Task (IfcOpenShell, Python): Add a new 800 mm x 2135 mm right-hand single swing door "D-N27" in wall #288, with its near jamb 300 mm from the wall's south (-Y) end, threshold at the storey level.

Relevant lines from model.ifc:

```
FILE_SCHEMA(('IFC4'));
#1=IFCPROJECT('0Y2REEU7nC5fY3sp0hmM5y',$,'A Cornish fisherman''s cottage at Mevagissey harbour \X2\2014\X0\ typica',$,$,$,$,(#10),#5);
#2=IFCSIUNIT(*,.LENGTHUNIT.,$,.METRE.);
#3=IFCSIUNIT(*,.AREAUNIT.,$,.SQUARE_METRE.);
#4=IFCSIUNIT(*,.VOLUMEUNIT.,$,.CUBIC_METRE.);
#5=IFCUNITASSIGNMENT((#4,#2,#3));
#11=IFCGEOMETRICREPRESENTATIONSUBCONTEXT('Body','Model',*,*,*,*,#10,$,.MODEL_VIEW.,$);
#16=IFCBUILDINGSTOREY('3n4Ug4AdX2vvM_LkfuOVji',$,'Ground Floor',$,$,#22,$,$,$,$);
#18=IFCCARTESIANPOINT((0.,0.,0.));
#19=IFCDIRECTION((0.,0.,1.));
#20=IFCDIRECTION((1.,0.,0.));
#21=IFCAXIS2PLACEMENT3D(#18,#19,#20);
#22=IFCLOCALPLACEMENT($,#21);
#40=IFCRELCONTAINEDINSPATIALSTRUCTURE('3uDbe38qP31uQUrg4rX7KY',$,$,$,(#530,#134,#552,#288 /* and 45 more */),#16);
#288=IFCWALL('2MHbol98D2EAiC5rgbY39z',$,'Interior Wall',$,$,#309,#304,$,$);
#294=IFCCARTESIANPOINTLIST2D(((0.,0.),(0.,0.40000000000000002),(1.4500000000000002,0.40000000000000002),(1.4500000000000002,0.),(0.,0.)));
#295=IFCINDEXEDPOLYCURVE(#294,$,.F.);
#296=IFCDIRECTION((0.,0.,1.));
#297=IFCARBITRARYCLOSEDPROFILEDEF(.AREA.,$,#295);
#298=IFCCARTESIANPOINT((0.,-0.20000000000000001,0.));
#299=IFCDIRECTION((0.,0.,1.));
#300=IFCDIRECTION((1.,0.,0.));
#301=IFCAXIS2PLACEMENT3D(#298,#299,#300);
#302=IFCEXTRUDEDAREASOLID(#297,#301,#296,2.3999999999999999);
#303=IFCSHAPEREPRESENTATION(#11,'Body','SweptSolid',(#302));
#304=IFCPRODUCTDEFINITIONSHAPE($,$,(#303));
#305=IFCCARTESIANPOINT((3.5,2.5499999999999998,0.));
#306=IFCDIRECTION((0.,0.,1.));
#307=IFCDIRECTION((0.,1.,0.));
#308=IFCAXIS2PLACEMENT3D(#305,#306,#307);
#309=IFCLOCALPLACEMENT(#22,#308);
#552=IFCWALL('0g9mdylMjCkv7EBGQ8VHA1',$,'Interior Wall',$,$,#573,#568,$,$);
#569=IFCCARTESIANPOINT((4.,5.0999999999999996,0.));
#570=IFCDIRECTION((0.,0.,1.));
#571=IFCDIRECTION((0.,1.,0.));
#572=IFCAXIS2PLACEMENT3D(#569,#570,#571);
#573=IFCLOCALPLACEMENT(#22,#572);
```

```python
import numpy as np
import ifcopenshell
import ifcopenshell.api.feature
import ifcopenshell.api.geometry
import ifcopenshell.api.root
import ifcopenshell.api.spatial
import ifcopenshell.geom
import ifcopenshell.util.element
import ifcopenshell.util.placement
import ifcopenshell.util.representation
import ifcopenshell.util.shape
import ifcopenshell.util.unit

model = ifcopenshell.open("model.ifc")
unit_scale = ifcopenshell.util.unit.calculate_unit_scale(model)
settings = ifcopenshell.geom.settings()


def volume(element):
    """Net volume in cubic metres, openings subtracted."""
    shape = ifcopenshell.geom.create_shape(settings, element)
    return ifcopenshell.util.shape.get_volume(shape.geometry)


wall = model.by_guid("2MHbol98D2EAiC5rgbY39z")
storey = ifcopenshell.util.element.get_container(wall, ifc_class="IfcBuildingStorey")
context = ifcopenshell.util.representation.get_context(model, "Model", "Body", "MODEL_VIEW")
before = volume(wall)

width, height, from_end, sill = 0.8, 2.135, 0.3, 0.0  # metres

# The wall runs along its own X axis, and the end named is its -X end.
wall_shape = ifcopenshell.geom.create_shape(settings, wall)
x, y, z = ifcopenshell.util.shape.get_vertices(wall_shape.geometry).T
start = x.min() + from_end
face, thickness = float(y.min()), float(y.max() - y.min())
wall_matrix = ifcopenshell.util.placement.get_local_placement(wall.ObjectPlacement)
level = ifcopenshell.util.placement.get_local_placement(storey.ObjectPlacement)[2, 3]


def in_wall(x, y):
    """Placement at x, y metres in the wall's axes, at sill height."""
    matrix = wall_matrix.copy()
    matrix[:, 3] = wall_matrix @ np.array([x / unit_scale, y / unit_scale, 0.0, 1.0])
    matrix[2, 3] = level + sill / unit_scale
    return matrix


# Opening: a box that overshoots both wall faces by 50 mm.
opening = ifcopenshell.api.root.create_entity(model, ifc_class="IfcOpeningElement", predefined_type="OPENING")
box = ifcopenshell.api.geometry.add_wall_representation(
    model, context=context, length=width, height=height, thickness=thickness + 0.1
)
ifcopenshell.api.geometry.assign_representation(model, product=opening, representation=box)
ifcopenshell.api.geometry.edit_object_placement(model, product=opening, matrix=in_wall(start, face - 0.05), is_si=False)
ifcopenshell.api.feature.add_feature(model, feature=opening, element=wall)

door = ifcopenshell.api.root.create_entity(model, ifc_class="IfcDoor", name="D-N27", predefined_type="DOOR")
door.OverallWidth, door.OverallHeight = width / unit_scale, height / unit_scale
door.OperationType = "SINGLE_SWING_RIGHT"
body = ifcopenshell.api.geometry.add_door_representation(
    model,
    context=context,
    overall_width=door.OverallWidth,
    overall_height=door.OverallHeight,
    operation_type="SINGLE_SWING_RIGHT",
    lining_properties={"LiningDepth": thickness / unit_scale, "ThresholdDepth": thickness / unit_scale},
)
ifcopenshell.api.geometry.assign_representation(model, product=door, representation=body)
ifcopenshell.api.spatial.assign_container(model, products=[door], relating_structure=storey)
ifcopenshell.api.feature.add_filling(model, opening=opening, element=door)

# The lining spans the wall, so the door starts at the wall face.
ifcopenshell.api.geometry.edit_object_placement(model, product=door, matrix=in_wall(start, face), is_si=False)

after = volume(wall)

print(f"wall volume {before:.3f} -> {after:.3f} m3")

model.write("model_updated.ifc")
```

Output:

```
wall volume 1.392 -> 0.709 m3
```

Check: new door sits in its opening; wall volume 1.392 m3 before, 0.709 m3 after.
